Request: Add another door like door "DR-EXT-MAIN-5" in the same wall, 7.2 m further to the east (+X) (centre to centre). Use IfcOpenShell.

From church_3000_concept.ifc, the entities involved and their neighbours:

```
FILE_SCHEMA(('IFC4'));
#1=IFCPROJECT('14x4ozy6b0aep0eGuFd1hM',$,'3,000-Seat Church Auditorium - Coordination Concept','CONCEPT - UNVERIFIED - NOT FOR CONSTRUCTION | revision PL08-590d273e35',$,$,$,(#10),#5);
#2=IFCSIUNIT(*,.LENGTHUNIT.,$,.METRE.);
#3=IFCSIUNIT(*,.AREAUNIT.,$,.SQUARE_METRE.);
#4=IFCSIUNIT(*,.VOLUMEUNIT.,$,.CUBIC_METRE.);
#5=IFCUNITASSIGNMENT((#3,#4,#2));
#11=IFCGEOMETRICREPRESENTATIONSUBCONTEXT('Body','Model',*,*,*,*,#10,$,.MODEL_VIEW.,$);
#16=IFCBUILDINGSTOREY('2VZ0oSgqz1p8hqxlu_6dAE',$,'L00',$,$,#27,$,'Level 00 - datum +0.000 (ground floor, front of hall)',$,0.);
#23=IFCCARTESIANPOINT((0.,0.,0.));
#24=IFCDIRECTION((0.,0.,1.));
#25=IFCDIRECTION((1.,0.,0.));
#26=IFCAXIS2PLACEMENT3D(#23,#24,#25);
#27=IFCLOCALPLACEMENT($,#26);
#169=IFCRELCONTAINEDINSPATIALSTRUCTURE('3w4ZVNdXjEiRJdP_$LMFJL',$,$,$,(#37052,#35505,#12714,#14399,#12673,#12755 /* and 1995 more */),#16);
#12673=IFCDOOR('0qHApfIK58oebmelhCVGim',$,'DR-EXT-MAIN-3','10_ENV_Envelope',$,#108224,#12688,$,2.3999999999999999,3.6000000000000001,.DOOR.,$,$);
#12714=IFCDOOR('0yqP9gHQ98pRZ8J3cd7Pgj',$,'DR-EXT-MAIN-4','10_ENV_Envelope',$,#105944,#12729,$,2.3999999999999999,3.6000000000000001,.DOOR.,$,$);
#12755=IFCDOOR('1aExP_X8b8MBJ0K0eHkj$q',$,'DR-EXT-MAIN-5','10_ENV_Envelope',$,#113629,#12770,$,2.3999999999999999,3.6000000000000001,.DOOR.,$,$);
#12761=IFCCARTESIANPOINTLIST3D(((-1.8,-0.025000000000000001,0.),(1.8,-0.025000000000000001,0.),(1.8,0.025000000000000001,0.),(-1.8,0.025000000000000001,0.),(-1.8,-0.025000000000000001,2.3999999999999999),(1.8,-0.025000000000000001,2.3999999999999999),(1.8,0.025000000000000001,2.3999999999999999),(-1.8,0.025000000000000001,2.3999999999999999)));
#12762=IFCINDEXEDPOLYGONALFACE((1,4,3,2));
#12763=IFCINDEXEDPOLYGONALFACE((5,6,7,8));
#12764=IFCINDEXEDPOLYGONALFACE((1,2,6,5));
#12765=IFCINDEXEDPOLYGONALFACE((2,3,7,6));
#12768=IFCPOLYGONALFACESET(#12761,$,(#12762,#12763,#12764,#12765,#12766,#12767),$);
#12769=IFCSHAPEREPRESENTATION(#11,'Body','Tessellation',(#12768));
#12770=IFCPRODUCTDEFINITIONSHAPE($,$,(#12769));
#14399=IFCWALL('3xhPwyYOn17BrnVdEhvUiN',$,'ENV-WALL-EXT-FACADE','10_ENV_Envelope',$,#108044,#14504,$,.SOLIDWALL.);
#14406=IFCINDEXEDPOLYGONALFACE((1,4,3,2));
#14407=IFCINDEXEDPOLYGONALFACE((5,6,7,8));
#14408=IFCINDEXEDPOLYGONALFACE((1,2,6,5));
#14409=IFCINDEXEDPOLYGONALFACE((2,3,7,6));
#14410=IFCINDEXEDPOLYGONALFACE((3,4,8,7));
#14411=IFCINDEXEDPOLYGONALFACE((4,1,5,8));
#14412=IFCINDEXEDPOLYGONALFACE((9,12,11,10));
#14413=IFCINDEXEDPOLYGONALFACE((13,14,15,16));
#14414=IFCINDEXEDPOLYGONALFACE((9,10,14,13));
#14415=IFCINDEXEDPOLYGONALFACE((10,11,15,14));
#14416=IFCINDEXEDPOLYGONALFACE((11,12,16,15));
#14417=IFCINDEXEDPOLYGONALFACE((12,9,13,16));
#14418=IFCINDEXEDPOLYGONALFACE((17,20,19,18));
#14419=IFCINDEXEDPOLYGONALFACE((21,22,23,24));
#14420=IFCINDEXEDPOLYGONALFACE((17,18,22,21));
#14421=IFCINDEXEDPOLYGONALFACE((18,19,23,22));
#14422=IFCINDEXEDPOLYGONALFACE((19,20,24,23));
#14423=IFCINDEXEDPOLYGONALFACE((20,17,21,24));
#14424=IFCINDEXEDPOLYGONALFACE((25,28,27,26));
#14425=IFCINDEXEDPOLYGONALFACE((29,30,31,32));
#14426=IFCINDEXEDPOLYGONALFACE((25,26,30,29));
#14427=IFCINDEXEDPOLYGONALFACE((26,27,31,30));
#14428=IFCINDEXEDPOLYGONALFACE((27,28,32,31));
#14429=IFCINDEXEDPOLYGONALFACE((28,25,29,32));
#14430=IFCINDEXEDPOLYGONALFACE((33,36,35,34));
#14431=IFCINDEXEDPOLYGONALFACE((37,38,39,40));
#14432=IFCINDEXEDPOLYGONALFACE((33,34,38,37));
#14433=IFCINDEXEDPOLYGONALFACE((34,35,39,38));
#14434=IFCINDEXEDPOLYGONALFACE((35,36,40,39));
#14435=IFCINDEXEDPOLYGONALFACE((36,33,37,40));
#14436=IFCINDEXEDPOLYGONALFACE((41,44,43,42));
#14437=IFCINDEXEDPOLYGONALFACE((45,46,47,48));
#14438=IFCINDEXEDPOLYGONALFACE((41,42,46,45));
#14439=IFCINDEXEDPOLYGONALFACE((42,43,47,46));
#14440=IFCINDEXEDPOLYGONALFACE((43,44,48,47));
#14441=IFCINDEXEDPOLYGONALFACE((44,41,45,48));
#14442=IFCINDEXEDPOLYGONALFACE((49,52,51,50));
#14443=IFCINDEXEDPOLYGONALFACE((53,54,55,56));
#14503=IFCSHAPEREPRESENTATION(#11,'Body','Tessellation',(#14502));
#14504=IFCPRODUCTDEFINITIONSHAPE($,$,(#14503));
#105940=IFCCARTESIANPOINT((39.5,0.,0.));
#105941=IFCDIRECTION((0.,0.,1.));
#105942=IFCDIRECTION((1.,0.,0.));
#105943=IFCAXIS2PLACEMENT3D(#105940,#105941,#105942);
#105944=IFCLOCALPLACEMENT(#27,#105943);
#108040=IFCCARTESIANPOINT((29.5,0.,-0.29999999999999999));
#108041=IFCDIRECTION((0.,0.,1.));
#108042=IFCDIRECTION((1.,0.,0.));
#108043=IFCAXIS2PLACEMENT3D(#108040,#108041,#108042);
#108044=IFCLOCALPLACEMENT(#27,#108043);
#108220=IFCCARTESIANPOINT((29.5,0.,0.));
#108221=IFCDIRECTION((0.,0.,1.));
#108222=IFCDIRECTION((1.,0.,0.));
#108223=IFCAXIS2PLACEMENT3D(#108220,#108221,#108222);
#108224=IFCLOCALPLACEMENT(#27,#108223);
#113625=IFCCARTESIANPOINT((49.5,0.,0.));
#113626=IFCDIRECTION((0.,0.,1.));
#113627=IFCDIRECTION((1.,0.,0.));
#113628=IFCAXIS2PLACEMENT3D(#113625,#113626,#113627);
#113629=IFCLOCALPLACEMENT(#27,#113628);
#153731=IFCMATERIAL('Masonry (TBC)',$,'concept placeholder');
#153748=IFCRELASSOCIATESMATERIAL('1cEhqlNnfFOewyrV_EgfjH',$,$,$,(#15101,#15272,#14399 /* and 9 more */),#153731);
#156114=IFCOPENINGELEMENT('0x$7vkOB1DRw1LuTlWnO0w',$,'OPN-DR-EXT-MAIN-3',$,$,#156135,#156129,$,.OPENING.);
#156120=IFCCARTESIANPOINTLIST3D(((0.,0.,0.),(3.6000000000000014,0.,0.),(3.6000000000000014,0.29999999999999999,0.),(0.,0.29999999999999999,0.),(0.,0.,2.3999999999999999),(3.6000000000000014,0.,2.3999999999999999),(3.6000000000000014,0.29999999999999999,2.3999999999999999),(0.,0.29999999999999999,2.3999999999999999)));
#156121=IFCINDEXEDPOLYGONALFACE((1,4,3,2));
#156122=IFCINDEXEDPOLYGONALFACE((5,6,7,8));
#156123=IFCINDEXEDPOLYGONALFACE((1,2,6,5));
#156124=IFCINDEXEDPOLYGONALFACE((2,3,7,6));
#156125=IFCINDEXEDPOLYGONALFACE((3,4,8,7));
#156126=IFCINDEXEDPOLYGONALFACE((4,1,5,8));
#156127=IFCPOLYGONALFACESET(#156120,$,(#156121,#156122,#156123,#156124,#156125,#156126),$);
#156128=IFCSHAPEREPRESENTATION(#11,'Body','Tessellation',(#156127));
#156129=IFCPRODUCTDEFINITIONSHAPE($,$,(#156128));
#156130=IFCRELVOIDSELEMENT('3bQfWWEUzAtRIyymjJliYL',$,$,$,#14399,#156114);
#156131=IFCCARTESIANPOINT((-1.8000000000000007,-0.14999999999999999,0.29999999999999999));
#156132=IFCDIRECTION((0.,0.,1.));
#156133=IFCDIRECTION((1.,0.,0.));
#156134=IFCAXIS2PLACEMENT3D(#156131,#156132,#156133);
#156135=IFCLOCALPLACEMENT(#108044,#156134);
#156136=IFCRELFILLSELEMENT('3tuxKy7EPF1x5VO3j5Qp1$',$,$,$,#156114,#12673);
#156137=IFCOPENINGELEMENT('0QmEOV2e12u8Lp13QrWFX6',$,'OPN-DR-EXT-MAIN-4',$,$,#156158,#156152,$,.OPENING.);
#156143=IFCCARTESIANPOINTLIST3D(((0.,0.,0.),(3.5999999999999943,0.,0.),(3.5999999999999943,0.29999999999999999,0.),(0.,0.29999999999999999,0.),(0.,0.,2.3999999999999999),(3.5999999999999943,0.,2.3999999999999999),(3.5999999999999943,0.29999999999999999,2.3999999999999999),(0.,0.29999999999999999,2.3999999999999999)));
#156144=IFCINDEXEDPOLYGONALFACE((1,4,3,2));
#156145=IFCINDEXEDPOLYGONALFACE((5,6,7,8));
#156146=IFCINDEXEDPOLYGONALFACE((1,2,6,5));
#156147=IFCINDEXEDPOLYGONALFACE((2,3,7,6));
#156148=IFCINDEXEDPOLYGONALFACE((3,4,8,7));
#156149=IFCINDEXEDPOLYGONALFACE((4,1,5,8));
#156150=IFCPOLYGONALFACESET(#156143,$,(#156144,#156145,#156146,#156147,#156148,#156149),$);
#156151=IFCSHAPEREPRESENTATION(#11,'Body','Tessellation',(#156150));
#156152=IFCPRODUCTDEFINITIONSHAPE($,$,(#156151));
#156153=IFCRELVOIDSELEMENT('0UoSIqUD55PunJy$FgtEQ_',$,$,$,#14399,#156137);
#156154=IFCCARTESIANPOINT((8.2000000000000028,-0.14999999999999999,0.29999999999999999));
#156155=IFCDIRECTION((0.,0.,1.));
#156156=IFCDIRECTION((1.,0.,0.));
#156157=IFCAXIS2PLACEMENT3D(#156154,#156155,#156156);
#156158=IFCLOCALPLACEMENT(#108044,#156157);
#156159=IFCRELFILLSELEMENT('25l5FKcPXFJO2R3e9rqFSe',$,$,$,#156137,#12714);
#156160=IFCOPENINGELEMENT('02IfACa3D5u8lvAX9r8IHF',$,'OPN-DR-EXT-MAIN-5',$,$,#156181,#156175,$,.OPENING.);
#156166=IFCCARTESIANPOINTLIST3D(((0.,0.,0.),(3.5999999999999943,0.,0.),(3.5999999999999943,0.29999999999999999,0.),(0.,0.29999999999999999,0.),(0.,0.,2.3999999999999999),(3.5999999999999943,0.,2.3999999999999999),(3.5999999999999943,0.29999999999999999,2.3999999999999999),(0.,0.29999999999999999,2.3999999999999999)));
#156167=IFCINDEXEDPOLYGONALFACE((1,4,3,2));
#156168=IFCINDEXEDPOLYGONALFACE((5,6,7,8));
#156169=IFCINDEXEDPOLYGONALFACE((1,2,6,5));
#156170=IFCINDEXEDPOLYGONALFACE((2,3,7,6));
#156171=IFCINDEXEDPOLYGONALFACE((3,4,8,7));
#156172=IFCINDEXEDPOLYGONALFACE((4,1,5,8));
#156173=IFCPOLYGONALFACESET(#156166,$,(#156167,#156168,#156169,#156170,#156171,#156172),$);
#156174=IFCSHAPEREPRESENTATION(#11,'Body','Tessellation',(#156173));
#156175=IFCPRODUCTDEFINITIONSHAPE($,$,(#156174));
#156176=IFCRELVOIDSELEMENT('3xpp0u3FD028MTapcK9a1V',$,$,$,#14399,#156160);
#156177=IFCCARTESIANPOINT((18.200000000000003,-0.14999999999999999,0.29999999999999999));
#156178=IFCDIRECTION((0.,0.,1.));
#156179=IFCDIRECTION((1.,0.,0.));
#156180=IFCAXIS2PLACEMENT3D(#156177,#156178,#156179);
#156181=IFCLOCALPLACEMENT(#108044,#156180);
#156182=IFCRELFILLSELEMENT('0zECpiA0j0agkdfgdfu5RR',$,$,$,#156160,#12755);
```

```python
import ifcopenshell
import ifcopenshell.api.feature
import ifcopenshell.api.geometry
import ifcopenshell.api.root
import ifcopenshell.geom
import ifcopenshell.util.element
import ifcopenshell.util.placement
import ifcopenshell.util.shape
import ifcopenshell.util.unit

model = ifcopenshell.open("church_3000_concept.ifc")
unit_scale = ifcopenshell.util.unit.calculate_unit_scale(model)
settings = ifcopenshell.geom.settings()


def volume(element):
    """Net volume in cubic metres, openings subtracted."""
    shape = ifcopenshell.geom.create_shape(settings, element)
    return ifcopenshell.util.shape.get_volume(shape.geometry)


door = model.by_guid("1aExP_X8b8MBJ0K0eHkj$q")
opening = door.FillsVoids[0].RelatingOpeningElement
wall = opening.VoidsElements[0].RelatingBuildingElement
before = volume(wall)
shift = ifcopenshell.util.placement.get_local_placement(wall.ObjectPlacement)[:3, 0] * 7.2 / unit_scale

# copy_class copies the void relationship, type, container and properties, but no geometry.
new_opening = ifcopenshell.api.root.copy_class(model, product=opening)
new_opening.Representation = ifcopenshell.util.element.copy_deep(
    model, opening.Representation, exclude=["IfcGeometricRepresentationContext", "IfcRepresentationMap"]
)
new_door = ifcopenshell.api.root.copy_class(model, product=door)
new_door.Representation = ifcopenshell.util.element.copy_deep(
    model, door.Representation, exclude=["IfcGeometricRepresentationContext", "IfcRepresentationMap"]
)
ifcopenshell.api.feature.add_filling(model, opening=new_opening, element=new_door)

for old, new in ((opening, new_opening), (door, new_door)):
    matrix = ifcopenshell.util.placement.get_local_placement(old.ObjectPlacement)
    matrix[:3, 3] += shift
    ifcopenshell.api.geometry.edit_object_placement(model, product=new, matrix=matrix, is_si=False)

after = volume(wall)

print(f"wall volume {before:.3f} -> {after:.3f} m3")

model.write("church_3000_concept_updated.ifc")
```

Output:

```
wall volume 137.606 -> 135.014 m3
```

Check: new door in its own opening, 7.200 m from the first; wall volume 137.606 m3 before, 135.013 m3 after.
